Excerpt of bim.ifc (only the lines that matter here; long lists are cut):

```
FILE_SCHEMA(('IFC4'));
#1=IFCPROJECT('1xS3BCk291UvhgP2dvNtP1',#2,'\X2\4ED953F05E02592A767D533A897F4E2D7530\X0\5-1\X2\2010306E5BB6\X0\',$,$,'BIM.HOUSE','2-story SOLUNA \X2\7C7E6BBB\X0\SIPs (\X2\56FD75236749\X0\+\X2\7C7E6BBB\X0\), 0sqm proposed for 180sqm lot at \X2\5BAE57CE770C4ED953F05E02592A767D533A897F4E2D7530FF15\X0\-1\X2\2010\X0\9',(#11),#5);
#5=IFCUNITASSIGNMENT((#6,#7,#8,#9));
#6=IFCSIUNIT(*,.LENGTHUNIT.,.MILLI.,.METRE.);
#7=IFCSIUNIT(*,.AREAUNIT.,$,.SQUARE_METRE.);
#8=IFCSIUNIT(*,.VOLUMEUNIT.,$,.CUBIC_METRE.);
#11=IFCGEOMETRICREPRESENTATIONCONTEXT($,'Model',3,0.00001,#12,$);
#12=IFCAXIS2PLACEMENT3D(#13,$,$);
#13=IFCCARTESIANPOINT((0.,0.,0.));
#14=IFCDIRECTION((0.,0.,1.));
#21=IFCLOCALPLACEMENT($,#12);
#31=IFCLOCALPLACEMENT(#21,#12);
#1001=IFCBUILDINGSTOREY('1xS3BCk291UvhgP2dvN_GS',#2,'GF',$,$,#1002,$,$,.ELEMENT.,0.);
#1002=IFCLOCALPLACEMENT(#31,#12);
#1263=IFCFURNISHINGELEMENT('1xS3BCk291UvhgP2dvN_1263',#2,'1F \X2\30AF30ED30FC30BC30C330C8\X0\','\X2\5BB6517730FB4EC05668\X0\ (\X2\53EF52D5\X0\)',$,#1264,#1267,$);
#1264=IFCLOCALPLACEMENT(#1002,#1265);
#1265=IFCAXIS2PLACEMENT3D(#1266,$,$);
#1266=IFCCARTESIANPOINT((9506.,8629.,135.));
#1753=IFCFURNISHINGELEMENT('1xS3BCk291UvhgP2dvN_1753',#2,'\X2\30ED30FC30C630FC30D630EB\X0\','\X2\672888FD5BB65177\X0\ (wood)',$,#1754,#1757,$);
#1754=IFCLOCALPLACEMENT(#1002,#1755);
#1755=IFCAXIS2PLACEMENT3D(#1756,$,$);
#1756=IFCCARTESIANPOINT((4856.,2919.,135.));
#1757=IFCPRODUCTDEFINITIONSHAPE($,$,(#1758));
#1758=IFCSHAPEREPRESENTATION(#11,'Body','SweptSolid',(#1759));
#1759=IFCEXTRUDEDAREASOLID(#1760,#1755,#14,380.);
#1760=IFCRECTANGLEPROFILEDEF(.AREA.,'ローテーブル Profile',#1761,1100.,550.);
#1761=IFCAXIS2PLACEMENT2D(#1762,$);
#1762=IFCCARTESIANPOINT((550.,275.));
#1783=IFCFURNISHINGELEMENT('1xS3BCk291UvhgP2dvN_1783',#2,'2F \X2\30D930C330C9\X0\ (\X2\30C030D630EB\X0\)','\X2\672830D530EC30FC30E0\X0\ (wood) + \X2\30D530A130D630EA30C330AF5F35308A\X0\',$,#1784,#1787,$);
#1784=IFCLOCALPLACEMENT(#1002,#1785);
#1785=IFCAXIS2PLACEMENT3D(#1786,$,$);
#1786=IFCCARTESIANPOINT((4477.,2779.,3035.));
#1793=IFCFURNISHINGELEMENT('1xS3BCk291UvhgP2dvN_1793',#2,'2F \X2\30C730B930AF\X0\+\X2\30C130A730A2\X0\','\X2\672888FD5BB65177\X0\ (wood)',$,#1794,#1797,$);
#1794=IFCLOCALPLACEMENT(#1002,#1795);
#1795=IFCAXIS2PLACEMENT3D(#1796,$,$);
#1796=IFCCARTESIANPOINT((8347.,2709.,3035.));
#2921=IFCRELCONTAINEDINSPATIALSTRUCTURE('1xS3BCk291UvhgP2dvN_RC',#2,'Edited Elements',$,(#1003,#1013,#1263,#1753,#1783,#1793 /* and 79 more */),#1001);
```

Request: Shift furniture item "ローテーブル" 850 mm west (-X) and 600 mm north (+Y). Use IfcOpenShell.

```python
import ifcopenshell
import ifcopenshell.api.geometry
import ifcopenshell.util.placement
import ifcopenshell.util.unit

model = ifcopenshell.open("bim.ifc")
unit_scale = ifcopenshell.util.unit.calculate_unit_scale(model)

item = model.by_id(1753)
matrix = ifcopenshell.util.placement.get_local_placement(item.ObjectPlacement)
matrix[0, 3] -= 0.85 / unit_scale
matrix[1, 3] += 0.6 / unit_scale
ifcopenshell.api.geometry.edit_object_placement(model, product=item, matrix=matrix, is_si=False)

print(ifcopenshell.util.placement.get_local_placement(item.ObjectPlacement).round(3) + 0.0)

model.write("bim_updated.ifc")
```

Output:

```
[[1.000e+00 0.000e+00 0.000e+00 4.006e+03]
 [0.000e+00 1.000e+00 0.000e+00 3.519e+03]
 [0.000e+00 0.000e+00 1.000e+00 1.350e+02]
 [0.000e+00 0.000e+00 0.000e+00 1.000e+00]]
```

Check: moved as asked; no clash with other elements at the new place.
